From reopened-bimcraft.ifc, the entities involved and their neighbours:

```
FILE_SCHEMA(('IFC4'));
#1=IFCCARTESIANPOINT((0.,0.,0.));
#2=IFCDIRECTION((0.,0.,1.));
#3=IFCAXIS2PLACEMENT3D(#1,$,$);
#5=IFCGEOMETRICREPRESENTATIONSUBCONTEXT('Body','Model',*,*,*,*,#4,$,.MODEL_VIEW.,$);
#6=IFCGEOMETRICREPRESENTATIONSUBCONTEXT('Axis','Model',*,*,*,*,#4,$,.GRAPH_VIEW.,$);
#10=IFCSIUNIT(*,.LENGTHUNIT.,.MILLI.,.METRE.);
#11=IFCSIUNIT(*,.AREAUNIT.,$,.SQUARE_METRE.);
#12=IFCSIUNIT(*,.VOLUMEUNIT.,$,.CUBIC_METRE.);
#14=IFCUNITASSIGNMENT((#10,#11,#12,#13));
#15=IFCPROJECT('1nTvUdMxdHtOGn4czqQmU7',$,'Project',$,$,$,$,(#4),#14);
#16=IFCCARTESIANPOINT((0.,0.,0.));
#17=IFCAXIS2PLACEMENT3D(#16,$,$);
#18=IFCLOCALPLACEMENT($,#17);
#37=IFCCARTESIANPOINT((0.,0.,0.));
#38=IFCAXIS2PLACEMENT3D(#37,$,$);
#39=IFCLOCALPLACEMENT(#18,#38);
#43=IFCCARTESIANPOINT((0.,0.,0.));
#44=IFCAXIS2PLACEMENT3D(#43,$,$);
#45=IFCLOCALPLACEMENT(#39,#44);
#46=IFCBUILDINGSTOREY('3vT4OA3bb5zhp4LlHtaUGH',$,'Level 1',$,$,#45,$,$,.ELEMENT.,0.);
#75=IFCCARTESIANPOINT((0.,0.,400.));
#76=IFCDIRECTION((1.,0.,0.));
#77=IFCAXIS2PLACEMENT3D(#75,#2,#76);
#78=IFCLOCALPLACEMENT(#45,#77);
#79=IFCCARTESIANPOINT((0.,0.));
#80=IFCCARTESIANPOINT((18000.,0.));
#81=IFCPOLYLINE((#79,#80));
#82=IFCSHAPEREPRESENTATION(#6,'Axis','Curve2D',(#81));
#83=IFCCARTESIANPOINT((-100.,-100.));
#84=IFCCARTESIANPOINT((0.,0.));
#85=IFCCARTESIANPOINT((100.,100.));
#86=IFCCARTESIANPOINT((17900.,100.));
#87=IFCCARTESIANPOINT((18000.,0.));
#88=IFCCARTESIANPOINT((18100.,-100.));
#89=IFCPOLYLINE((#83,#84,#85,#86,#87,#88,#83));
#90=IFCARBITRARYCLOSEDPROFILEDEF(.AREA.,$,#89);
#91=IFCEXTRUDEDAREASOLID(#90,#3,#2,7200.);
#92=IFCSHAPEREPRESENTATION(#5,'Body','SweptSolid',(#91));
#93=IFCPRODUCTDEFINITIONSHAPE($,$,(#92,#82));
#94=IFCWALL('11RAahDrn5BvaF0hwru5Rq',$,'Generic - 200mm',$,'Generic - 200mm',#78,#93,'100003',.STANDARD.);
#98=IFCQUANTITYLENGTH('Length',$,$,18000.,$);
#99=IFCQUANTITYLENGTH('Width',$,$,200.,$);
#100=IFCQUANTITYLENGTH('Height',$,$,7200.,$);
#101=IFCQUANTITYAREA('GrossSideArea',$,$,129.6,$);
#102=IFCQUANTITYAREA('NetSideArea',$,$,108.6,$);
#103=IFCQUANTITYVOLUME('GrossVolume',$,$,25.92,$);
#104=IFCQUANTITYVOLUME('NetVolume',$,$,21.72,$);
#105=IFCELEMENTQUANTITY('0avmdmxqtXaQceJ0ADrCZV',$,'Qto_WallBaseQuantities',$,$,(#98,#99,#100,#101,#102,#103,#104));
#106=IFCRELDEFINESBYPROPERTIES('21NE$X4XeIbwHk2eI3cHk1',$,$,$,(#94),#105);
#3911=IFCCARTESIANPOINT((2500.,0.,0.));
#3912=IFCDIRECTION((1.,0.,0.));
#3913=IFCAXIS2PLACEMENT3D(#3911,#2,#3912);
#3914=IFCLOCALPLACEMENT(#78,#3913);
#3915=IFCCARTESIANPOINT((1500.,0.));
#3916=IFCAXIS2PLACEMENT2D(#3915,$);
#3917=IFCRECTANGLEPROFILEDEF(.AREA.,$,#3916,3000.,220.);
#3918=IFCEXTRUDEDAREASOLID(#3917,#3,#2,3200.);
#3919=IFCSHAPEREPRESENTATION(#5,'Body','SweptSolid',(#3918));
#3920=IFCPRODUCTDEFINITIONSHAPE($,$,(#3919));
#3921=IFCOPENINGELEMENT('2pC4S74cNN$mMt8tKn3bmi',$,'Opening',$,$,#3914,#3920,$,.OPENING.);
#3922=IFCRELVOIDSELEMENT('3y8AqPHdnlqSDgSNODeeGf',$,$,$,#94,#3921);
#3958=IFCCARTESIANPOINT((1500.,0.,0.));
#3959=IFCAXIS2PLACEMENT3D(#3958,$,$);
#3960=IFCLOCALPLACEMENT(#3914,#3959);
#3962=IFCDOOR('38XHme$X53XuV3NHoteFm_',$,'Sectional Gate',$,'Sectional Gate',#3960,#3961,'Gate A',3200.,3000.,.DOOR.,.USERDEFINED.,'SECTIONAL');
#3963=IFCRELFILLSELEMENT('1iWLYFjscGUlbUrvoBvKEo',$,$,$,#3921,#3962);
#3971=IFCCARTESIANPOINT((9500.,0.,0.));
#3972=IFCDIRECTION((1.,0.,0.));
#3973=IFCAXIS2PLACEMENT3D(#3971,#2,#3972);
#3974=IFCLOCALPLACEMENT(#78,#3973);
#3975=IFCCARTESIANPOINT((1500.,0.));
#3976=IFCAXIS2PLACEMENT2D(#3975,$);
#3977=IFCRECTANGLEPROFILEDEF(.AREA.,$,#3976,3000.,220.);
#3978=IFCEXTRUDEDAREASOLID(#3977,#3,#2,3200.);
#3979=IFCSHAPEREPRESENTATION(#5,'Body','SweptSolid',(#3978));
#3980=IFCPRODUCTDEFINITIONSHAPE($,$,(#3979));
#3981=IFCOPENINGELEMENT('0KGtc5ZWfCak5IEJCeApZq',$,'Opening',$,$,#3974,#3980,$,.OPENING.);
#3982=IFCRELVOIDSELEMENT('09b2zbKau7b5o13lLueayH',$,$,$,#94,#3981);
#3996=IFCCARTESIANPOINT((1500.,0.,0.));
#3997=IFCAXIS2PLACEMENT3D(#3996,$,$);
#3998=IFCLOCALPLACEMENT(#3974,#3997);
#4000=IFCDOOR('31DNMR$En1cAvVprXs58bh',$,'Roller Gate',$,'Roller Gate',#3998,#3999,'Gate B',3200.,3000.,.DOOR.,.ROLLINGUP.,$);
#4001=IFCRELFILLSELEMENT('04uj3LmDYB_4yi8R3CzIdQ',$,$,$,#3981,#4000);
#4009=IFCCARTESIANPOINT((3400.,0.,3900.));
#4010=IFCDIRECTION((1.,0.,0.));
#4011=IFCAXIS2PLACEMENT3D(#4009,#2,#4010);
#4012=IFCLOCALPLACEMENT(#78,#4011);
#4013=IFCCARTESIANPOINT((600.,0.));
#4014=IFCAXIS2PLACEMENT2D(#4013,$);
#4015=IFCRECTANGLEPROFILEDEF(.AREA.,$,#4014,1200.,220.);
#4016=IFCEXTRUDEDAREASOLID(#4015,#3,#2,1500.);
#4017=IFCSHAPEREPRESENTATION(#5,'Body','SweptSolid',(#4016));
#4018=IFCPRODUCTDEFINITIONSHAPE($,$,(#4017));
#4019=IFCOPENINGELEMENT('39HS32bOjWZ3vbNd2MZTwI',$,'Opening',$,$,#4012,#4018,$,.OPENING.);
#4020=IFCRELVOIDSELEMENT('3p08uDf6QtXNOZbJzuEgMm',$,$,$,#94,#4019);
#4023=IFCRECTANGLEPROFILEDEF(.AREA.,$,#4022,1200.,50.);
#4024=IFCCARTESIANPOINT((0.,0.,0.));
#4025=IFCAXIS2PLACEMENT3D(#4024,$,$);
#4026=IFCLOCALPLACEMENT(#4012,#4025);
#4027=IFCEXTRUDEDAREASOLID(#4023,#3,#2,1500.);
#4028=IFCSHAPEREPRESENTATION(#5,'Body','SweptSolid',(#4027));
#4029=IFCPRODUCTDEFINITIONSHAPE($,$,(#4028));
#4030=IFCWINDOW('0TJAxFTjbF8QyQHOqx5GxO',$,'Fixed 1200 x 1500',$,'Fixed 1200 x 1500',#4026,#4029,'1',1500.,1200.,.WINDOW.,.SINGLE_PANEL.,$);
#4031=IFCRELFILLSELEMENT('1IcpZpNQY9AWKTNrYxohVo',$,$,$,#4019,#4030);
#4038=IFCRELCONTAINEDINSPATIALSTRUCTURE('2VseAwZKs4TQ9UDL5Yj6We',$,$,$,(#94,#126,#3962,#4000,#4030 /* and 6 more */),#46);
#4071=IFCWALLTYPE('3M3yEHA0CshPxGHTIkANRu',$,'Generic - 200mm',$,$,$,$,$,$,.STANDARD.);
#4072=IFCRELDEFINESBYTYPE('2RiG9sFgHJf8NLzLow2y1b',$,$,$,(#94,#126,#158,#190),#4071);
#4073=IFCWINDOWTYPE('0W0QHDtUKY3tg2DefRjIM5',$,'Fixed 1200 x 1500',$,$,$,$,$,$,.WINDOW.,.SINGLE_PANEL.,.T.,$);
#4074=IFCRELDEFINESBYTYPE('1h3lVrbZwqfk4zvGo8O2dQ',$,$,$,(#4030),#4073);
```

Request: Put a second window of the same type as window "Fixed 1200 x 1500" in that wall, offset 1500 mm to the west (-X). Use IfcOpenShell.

```python
import ifcopenshell
import ifcopenshell.api.feature
import ifcopenshell.api.geometry
import ifcopenshell.api.pset
import ifcopenshell.api.root
import ifcopenshell.geom
import ifcopenshell.util.element
import ifcopenshell.util.placement
import ifcopenshell.util.shape
import ifcopenshell.util.unit

model = ifcopenshell.open("reopened-bimcraft.ifc")
area_scale = ifcopenshell.util.unit.calculate_unit_scale(model, "AREAUNIT")
volume_scale = ifcopenshell.util.unit.calculate_unit_scale(model, "VOLUMEUNIT")
settings = ifcopenshell.geom.settings()


def volume(element):
    """Net volume in cubic metres, openings subtracted."""
    shape = ifcopenshell.geom.create_shape(settings, element)
    return ifcopenshell.util.shape.get_volume(shape.geometry)


window = model.by_id(4030)
opening = window.FillsVoids[0].RelatingOpeningElement
wall = opening.VoidsElements[0].RelatingBuildingElement
before = volume(wall)
shift = ifcopenshell.util.placement.get_local_placement(wall.ObjectPlacement)[:3, 0] * -1500.0

# copy_class copies the void relationship, type, container and properties, but no geometry.
new_opening = ifcopenshell.api.root.copy_class(model, product=opening)
new_opening.Representation = ifcopenshell.util.element.copy_deep(
    model, opening.Representation, exclude=["IfcGeometricRepresentationContext", "IfcRepresentationMap"]
)
new_window = ifcopenshell.api.root.copy_class(model, product=window)
new_window.Representation = ifcopenshell.util.element.copy_deep(
    model, window.Representation, exclude=["IfcGeometricRepresentationContext", "IfcRepresentationMap"]
)
new_window.Tag = None
ifcopenshell.api.feature.add_filling(model, opening=new_opening, element=new_window)

for old, new in ((opening, new_opening), (window, new_window)):
    matrix = ifcopenshell.util.placement.get_local_placement(old.ObjectPlacement)
    matrix[:3, 3] += shift
    ifcopenshell.api.geometry.edit_object_placement(model, product=new, matrix=matrix, is_si=False)

after = volume(wall)
thickness = 0.2  # wall thickness in metres

# Update the wall's stored quantities.
qto = model.by_id(ifcopenshell.util.element.get_pset(wall, "Qto_WallBaseQuantities", should_inherit=False)["id"])
ifcopenshell.api.pset.edit_qto(model, qto=qto, properties={
    "NetSideArea": after / thickness / area_scale,
    "NetVolume": after / volume_scale,
})

print(f"wall volume {before:.3f} -> {after:.3f} m3")

model.write("reopened-bimcraft_updated.ifc")
```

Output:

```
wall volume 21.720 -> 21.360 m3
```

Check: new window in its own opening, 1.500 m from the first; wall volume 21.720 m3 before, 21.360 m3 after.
